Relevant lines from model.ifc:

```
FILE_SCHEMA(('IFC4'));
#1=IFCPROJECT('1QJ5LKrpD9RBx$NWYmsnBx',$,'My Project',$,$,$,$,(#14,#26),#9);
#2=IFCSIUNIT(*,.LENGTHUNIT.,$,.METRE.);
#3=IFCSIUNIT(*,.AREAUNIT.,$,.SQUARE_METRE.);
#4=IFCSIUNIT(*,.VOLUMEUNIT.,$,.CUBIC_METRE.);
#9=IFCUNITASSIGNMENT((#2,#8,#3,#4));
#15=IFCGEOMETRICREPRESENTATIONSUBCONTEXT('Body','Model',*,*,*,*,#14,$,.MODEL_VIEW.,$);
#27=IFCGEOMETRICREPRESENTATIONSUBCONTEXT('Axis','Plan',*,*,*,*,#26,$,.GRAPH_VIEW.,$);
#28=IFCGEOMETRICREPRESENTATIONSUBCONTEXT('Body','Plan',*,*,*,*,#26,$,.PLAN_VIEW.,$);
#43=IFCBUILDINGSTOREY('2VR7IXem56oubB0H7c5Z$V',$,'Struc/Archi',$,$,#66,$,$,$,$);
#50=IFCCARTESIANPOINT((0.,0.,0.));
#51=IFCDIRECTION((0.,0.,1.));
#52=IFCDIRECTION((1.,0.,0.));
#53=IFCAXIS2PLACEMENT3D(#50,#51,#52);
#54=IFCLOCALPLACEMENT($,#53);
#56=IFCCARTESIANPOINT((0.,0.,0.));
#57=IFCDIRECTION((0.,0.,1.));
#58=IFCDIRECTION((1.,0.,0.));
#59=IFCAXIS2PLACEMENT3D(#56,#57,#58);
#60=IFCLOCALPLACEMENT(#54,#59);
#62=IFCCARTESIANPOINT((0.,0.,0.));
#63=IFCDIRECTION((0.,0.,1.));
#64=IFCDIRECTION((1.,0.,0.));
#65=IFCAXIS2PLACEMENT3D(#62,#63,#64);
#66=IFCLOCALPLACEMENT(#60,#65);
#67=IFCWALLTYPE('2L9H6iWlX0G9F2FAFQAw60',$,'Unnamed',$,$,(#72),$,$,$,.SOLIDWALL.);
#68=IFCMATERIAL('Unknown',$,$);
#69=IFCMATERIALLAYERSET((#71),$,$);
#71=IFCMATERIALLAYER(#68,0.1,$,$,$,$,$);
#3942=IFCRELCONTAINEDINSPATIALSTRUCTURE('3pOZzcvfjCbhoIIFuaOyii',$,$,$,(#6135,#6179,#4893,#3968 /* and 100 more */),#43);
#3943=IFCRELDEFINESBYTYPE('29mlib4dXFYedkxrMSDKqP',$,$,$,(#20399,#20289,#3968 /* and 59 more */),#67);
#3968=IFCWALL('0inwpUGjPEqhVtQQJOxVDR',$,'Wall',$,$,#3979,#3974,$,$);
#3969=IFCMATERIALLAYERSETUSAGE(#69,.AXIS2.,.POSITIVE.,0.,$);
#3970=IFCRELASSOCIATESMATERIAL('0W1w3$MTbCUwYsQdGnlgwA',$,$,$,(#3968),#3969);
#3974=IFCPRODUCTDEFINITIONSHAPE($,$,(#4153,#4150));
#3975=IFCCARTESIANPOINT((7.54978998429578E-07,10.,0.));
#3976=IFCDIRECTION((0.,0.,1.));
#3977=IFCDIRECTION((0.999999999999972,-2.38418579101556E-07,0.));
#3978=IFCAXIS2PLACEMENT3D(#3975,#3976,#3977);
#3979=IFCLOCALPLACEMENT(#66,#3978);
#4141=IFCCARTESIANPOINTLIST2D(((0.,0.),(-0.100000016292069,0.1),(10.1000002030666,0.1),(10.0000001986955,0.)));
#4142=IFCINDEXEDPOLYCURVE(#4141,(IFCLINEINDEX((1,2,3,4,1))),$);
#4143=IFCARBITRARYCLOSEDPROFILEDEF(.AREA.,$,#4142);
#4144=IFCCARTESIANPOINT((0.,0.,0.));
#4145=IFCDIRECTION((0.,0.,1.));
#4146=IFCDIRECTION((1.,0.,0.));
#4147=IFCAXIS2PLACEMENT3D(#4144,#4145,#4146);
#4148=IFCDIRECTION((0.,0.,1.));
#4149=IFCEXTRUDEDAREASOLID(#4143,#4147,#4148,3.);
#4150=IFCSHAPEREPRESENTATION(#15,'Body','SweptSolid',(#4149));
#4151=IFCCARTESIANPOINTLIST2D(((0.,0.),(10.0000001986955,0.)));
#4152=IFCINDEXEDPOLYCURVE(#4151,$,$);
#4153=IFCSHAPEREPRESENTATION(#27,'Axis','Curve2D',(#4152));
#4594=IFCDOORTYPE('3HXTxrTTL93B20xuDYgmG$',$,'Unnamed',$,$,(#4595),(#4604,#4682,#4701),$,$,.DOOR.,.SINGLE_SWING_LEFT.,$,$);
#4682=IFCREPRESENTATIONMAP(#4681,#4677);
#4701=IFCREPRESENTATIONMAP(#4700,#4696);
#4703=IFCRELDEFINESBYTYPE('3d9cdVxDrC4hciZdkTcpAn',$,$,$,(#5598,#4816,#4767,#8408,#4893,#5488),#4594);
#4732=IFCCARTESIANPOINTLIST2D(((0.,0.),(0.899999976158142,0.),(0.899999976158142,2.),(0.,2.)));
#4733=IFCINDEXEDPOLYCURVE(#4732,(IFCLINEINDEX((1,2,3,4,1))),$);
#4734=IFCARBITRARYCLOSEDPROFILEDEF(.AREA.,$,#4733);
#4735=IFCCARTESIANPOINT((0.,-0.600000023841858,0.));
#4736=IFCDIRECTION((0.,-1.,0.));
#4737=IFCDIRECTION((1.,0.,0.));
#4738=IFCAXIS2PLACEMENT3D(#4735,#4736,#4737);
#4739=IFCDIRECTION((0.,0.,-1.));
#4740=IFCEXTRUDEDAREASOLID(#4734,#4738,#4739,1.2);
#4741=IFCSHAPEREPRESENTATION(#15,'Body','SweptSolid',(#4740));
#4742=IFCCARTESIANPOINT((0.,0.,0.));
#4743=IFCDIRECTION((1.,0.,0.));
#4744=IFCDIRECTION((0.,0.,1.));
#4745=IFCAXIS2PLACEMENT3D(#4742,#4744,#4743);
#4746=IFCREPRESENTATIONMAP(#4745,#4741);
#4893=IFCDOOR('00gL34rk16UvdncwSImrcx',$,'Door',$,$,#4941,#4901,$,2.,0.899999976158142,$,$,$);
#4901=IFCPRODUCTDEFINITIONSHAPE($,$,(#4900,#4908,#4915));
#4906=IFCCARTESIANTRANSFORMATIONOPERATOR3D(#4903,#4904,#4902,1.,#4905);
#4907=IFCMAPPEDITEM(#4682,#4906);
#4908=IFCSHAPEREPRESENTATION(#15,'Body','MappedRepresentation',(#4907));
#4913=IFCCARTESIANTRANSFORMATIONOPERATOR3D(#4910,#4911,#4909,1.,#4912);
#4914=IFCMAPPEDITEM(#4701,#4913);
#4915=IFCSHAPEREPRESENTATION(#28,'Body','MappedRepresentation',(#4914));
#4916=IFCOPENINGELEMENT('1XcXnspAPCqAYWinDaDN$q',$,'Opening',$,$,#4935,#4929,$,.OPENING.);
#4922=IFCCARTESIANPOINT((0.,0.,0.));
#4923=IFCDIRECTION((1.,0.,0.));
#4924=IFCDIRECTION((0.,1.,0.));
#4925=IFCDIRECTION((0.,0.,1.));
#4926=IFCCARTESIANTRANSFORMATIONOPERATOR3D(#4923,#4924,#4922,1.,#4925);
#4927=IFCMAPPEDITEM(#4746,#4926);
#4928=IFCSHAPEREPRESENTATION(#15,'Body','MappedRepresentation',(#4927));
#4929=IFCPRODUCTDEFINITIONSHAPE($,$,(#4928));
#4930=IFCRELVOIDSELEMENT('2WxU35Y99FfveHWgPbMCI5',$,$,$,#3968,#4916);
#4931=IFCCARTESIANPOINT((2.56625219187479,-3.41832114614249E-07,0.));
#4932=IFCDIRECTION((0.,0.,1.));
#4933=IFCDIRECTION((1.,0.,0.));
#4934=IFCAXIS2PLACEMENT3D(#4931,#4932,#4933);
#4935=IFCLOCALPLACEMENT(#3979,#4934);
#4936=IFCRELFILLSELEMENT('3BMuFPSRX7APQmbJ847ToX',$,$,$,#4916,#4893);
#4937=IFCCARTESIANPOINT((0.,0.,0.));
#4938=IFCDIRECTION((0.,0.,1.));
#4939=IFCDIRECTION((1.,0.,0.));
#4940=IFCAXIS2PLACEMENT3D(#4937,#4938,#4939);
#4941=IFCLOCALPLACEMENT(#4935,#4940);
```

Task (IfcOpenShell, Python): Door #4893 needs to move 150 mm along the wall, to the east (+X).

```python
import ifcopenshell
import ifcopenshell.api.geometry
import ifcopenshell.util.placement
import ifcopenshell.util.unit

model = ifcopenshell.open("model.ifc")
unit_scale = ifcopenshell.util.unit.calculate_unit_scale(model)

door = model.by_guid("00gL34rk16UvdncwSImrcx")
opening = door.FillsVoids[0].RelatingOpeningElement
wall = opening.VoidsElements[0].RelatingBuildingElement

wall_matrix = ifcopenshell.util.placement.get_local_placement(wall.ObjectPlacement)
shift = wall_matrix[:3, 0] * 0.15 / unit_scale
before = ifcopenshell.util.placement.get_local_placement(door.ObjectPlacement)[:3, 3].copy()

# The door is placed relative to its opening, so it follows when the opening moves.
matrix = ifcopenshell.util.placement.get_local_placement(opening.ObjectPlacement)
matrix[:3, 3] += shift
ifcopenshell.api.geometry.edit_object_placement(
    model, product=opening, matrix=matrix, is_si=False, should_transform_children=True
)

after = ifcopenshell.util.placement.get_local_placement(door.ObjectPlacement)[:3, 3]
print("door moved by", (after - before).round(3) + 0.0)

model.write("model_edited.ifc")
```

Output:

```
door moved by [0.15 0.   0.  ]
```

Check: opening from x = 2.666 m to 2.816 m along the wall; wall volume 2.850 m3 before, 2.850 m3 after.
